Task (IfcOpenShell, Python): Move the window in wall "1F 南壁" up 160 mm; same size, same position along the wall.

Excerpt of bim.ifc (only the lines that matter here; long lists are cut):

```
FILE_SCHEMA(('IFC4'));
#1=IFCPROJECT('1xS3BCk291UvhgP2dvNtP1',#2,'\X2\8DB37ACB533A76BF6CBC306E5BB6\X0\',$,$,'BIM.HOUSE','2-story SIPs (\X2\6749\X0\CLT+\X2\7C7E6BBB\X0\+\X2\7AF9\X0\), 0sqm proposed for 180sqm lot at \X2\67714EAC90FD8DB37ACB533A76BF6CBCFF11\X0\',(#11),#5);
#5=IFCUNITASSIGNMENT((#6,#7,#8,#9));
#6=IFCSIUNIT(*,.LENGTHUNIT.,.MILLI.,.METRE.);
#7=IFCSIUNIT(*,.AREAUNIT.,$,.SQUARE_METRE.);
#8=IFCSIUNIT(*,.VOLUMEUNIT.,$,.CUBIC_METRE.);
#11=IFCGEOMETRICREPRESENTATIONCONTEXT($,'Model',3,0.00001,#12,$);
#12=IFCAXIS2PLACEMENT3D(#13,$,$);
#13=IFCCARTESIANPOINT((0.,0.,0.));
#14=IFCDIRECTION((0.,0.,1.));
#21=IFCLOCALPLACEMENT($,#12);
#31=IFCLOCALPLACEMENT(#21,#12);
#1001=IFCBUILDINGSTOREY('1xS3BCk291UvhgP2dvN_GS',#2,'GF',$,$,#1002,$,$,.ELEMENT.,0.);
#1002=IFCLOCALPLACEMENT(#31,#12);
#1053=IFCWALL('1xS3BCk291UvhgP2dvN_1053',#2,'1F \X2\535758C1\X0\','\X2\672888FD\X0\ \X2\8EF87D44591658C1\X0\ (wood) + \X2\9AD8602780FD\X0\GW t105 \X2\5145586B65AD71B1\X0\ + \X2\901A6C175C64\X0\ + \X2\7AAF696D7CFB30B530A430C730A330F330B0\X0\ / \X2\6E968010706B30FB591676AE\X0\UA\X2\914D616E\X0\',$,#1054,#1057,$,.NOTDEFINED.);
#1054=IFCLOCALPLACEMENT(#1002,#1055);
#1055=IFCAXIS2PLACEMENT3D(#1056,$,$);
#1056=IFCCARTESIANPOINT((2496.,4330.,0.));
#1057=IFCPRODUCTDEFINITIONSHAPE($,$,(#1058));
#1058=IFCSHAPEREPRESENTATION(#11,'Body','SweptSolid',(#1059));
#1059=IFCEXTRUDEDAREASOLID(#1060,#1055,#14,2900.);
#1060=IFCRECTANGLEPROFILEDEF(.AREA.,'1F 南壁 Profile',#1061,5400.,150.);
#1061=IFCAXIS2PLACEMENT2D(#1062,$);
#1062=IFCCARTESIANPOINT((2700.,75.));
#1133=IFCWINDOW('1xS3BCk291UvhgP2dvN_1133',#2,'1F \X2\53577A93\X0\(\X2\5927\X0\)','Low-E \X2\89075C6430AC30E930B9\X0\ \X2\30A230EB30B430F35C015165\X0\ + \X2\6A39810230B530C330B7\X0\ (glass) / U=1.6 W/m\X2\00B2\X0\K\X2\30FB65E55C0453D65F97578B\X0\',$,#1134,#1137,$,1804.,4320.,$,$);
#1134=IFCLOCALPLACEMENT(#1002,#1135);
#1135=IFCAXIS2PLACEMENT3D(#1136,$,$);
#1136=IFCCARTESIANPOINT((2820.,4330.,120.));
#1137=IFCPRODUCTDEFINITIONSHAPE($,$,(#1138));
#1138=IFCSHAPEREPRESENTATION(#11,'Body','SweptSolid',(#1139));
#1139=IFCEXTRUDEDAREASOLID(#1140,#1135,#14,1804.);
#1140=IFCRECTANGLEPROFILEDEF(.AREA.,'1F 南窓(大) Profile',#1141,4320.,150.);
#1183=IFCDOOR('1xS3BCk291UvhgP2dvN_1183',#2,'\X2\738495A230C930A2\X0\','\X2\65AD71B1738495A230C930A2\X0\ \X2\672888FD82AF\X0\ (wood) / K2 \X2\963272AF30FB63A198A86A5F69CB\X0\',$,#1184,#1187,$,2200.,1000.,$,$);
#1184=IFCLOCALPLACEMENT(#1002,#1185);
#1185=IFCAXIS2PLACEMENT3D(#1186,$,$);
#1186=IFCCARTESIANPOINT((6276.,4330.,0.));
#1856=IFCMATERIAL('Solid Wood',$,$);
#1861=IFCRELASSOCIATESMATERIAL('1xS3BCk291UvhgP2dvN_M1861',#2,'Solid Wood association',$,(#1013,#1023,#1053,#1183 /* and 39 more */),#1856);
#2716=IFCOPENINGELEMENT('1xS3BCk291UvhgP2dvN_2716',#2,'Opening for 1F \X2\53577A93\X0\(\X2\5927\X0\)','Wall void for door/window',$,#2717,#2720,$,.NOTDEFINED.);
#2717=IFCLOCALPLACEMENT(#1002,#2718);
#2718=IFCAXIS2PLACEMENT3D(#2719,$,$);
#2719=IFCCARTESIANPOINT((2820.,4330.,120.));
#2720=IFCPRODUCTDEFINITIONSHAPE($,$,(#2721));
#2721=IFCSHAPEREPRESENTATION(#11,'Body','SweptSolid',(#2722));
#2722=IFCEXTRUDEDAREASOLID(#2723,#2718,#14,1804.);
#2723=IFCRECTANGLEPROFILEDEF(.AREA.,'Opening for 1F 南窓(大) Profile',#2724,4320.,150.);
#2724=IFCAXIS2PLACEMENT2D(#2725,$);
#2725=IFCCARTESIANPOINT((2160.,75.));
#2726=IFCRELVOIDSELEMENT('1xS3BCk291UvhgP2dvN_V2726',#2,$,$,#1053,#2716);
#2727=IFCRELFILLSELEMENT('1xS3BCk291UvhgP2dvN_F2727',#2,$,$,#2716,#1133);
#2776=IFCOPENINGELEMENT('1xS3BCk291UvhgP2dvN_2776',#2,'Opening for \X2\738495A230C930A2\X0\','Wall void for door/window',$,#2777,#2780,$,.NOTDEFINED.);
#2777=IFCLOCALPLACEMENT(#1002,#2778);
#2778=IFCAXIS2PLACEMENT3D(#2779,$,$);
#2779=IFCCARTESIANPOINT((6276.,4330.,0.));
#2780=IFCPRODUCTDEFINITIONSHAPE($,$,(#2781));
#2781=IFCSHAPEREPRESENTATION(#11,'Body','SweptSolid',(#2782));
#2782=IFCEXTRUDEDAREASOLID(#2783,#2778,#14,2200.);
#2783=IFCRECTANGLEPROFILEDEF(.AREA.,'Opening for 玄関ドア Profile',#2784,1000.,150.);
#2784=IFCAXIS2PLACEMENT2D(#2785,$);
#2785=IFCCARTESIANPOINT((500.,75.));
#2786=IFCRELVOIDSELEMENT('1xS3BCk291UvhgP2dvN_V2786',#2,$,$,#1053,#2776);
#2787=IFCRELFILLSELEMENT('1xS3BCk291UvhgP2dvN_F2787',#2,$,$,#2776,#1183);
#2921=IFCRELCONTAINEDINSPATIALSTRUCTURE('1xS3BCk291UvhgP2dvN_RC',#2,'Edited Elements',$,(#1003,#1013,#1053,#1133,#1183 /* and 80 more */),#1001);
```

```python
import numpy as np
import ifcopenshell
import ifcopenshell.api.geometry
import ifcopenshell.util.placement
import ifcopenshell.util.unit

model = ifcopenshell.open("bim.ifc")
unit_scale = ifcopenshell.util.unit.calculate_unit_scale(model)

window = model.by_id(1133)
opening = window.FillsVoids[0].RelatingOpeningElement
dz = 160.0

shift = np.array([0.0, 0.0, dz])
# The window is not placed relative to its opening, so move both.
for product in (opening, window):
    matrix = ifcopenshell.util.placement.get_local_placement(product.ObjectPlacement)
    matrix[:3, 3] += shift
    ifcopenshell.api.geometry.edit_object_placement(model, product=product, matrix=matrix, is_si=False)

print(f"moved by {dz * unit_scale:+.3f} m")

model.write("bim_v2.ifc")
```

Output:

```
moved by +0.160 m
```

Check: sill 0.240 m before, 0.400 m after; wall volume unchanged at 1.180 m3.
